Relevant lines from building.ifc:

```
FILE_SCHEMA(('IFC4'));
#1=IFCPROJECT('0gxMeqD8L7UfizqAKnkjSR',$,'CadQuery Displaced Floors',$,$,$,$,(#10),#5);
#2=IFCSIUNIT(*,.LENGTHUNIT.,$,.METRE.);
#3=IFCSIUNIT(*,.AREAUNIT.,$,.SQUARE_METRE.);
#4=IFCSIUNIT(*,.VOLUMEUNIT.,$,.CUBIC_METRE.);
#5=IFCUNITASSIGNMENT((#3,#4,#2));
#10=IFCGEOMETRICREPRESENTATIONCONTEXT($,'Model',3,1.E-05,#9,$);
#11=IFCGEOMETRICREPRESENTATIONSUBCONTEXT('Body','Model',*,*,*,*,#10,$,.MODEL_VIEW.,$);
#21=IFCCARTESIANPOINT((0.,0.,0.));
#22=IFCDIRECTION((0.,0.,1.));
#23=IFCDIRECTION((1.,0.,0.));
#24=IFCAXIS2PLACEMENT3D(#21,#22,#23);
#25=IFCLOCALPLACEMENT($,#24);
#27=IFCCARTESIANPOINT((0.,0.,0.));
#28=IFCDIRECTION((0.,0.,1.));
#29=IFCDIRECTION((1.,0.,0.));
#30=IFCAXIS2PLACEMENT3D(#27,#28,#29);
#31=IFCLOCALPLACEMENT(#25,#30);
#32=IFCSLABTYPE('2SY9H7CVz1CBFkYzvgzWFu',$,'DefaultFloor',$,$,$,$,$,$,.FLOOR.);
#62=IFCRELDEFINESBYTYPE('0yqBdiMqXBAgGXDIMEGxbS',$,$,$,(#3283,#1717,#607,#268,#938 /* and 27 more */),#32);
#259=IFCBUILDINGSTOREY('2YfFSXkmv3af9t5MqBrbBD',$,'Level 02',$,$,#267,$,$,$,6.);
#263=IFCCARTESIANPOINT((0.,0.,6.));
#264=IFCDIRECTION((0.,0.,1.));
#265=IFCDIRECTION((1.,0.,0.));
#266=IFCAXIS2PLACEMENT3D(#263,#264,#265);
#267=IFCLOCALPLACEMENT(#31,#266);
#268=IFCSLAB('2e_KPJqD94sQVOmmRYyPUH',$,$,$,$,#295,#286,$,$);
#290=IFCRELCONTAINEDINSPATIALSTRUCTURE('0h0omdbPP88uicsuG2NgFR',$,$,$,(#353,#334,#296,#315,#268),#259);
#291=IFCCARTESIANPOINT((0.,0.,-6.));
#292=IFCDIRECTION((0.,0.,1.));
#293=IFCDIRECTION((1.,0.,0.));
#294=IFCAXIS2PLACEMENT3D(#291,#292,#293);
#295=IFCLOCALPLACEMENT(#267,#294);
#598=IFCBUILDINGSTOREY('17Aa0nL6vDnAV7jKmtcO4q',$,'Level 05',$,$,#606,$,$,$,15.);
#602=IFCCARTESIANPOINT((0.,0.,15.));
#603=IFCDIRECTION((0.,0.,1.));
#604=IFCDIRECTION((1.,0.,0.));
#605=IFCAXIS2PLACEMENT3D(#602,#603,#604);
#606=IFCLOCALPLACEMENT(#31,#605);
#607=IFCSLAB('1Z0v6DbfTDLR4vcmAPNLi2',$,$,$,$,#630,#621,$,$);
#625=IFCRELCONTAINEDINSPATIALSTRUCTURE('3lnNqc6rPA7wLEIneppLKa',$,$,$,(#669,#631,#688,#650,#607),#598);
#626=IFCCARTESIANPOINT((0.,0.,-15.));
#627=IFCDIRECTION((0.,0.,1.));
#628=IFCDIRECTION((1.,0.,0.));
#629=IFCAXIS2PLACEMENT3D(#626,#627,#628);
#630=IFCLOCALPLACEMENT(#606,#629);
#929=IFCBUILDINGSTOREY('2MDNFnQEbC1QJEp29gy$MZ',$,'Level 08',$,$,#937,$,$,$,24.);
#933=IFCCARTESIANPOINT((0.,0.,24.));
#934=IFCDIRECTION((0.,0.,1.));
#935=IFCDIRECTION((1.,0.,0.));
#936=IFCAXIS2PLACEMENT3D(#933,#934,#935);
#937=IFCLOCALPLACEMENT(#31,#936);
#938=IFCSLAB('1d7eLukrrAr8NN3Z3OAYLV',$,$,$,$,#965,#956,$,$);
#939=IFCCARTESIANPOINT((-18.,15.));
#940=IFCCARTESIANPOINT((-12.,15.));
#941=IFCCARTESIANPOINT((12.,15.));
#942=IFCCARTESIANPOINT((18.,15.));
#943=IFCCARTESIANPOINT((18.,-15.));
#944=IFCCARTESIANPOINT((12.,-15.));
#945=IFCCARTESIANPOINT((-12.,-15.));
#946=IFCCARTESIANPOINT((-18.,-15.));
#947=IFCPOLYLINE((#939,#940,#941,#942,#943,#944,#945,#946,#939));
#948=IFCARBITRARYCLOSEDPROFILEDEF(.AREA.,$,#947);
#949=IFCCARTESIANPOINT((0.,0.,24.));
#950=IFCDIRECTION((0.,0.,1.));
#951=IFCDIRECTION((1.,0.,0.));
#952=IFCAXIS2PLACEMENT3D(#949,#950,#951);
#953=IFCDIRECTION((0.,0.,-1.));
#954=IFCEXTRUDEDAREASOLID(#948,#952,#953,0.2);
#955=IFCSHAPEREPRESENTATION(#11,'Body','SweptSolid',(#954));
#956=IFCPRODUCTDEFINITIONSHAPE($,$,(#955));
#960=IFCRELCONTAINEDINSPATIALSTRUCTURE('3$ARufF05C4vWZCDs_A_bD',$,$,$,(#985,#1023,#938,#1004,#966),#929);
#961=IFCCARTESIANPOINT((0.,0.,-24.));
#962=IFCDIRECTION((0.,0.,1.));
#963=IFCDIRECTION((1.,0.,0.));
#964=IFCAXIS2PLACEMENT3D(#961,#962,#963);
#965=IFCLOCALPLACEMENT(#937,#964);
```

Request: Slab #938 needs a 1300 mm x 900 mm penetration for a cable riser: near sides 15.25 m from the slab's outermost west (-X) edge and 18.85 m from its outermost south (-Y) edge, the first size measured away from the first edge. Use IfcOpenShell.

```python
import numpy as np
import ifcopenshell
import ifcopenshell.api.feature
import ifcopenshell.api.geometry
import ifcopenshell.api.root
import ifcopenshell.geom
import ifcopenshell.util.placement
import ifcopenshell.util.representation
import ifcopenshell.util.shape
import ifcopenshell.util.unit

model = ifcopenshell.open("building.ifc")
unit_scale = ifcopenshell.util.unit.calculate_unit_scale(model)
settings = ifcopenshell.geom.settings()


def volume(element):
    """Net volume in cubic metres, openings subtracted."""
    shape = ifcopenshell.geom.create_shape(settings, element)
    return ifcopenshell.util.shape.get_volume(shape.geometry)


slab = model.by_guid("1d7eLukrrAr8NN3Z3OAYLV")
before = volume(slab)

# Extent in the slab's own axes, in metres. The edges named are its -X and -Y sides.
slab_shape = ifcopenshell.geom.create_shape(settings, slab)
vertices = ifcopenshell.util.shape.get_vertices(slab_shape.geometry)
x_min, y_min, bottom = vertices.min(axis=0)
top = vertices[:, 2].max()

opening = ifcopenshell.api.root.create_entity(model, ifc_class="IfcOpeningElement", name="Cable riser opening", predefined_type="OPENING")
context = ifcopenshell.util.representation.get_context(model, "Model", "Body", "MODEL_VIEW")
width, depth = 1.3, 0.9
outline = [(0.0, 0.0), (width, 0.0), (width, depth), (0.0, depth), (0.0, 0.0)]
# Overshoot both faces by 50 mm so the cut is clean.
shape = ifcopenshell.api.geometry.add_slab_representation(
    model, context=context, depth=top - bottom + 0.1, polyline=outline
)
ifcopenshell.api.geometry.assign_representation(model, product=opening, representation=shape)

matrix = ifcopenshell.util.placement.get_local_placement(slab.ObjectPlacement)
matrix[:, 3] = matrix @ np.append(np.array([x_min + 15.25, y_min + 18.85, bottom - 0.05]) / unit_scale, 1.0)
ifcopenshell.api.geometry.edit_object_placement(model, product=opening, matrix=matrix, is_si=False)
ifcopenshell.api.feature.add_feature(model, feature=opening, element=slab)

after = volume(slab)

print(f"slab volume {before:.3f} -> {after:.3f} m3")

model.write("building_updated.ifc")
```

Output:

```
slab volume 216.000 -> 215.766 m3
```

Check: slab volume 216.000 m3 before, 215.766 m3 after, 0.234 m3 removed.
